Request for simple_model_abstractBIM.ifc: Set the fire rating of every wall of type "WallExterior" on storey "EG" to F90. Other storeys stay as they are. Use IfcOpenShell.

First a look at what the model holds.

```python
import ifcopenshell
import ifcopenshell.util.element

model = ifcopenshell.open("simple_model_abstractBIM.ifc")
print(model.schema)
storey = next(s for s in model.by_type("IfcBuildingStorey") if s.Name == "EG")
walls = [e for e in ifcopenshell.util.element.get_decomposition(storey) if e.is_a("IfcWall")]
seen = {}
for e in walls:
    element_type = ifcopenshell.util.element.get_type(e)
    key = (element_type.Name if element_type != e and element_type else None, ifcopenshell.util.element.get_pset(e, "Pset_WallCommon", "FireRating"))
    seen[key] = seen.get(key, 0) + 1
for (name, value), count in sorted(seen.items(), key=str):
    print(count, "x", name, "|", value)
```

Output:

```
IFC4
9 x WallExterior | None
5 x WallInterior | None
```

```python
import ifcopenshell
import ifcopenshell.api.pset
import ifcopenshell.util.element

model = ifcopenshell.open("simple_model_abstractBIM.ifc")

storey = next(s for s in model.by_type("IfcBuildingStorey") if s.Name == "EG")
walls = [e for e in ifcopenshell.util.element.get_decomposition(storey) if e.is_a("IfcWall")]

count = 0
for e in walls:
    element_type = ifcopenshell.util.element.get_type(e)
    if element_type in (None, e) or element_type.Name != "WallExterior":
        continue
    # add_pset returns the element's existing set when there is one.
    pset = ifcopenshell.api.pset.add_pset(model, product=e, name="Pset_WallCommon")
    ifcopenshell.api.pset.edit_pset(model, pset=pset, properties={"FireRating": "F90"})
    count += 1

print(count, "walls updated")

model.write("simple_model_abstractBIM_updated.ifc")
```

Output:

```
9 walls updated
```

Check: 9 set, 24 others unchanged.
